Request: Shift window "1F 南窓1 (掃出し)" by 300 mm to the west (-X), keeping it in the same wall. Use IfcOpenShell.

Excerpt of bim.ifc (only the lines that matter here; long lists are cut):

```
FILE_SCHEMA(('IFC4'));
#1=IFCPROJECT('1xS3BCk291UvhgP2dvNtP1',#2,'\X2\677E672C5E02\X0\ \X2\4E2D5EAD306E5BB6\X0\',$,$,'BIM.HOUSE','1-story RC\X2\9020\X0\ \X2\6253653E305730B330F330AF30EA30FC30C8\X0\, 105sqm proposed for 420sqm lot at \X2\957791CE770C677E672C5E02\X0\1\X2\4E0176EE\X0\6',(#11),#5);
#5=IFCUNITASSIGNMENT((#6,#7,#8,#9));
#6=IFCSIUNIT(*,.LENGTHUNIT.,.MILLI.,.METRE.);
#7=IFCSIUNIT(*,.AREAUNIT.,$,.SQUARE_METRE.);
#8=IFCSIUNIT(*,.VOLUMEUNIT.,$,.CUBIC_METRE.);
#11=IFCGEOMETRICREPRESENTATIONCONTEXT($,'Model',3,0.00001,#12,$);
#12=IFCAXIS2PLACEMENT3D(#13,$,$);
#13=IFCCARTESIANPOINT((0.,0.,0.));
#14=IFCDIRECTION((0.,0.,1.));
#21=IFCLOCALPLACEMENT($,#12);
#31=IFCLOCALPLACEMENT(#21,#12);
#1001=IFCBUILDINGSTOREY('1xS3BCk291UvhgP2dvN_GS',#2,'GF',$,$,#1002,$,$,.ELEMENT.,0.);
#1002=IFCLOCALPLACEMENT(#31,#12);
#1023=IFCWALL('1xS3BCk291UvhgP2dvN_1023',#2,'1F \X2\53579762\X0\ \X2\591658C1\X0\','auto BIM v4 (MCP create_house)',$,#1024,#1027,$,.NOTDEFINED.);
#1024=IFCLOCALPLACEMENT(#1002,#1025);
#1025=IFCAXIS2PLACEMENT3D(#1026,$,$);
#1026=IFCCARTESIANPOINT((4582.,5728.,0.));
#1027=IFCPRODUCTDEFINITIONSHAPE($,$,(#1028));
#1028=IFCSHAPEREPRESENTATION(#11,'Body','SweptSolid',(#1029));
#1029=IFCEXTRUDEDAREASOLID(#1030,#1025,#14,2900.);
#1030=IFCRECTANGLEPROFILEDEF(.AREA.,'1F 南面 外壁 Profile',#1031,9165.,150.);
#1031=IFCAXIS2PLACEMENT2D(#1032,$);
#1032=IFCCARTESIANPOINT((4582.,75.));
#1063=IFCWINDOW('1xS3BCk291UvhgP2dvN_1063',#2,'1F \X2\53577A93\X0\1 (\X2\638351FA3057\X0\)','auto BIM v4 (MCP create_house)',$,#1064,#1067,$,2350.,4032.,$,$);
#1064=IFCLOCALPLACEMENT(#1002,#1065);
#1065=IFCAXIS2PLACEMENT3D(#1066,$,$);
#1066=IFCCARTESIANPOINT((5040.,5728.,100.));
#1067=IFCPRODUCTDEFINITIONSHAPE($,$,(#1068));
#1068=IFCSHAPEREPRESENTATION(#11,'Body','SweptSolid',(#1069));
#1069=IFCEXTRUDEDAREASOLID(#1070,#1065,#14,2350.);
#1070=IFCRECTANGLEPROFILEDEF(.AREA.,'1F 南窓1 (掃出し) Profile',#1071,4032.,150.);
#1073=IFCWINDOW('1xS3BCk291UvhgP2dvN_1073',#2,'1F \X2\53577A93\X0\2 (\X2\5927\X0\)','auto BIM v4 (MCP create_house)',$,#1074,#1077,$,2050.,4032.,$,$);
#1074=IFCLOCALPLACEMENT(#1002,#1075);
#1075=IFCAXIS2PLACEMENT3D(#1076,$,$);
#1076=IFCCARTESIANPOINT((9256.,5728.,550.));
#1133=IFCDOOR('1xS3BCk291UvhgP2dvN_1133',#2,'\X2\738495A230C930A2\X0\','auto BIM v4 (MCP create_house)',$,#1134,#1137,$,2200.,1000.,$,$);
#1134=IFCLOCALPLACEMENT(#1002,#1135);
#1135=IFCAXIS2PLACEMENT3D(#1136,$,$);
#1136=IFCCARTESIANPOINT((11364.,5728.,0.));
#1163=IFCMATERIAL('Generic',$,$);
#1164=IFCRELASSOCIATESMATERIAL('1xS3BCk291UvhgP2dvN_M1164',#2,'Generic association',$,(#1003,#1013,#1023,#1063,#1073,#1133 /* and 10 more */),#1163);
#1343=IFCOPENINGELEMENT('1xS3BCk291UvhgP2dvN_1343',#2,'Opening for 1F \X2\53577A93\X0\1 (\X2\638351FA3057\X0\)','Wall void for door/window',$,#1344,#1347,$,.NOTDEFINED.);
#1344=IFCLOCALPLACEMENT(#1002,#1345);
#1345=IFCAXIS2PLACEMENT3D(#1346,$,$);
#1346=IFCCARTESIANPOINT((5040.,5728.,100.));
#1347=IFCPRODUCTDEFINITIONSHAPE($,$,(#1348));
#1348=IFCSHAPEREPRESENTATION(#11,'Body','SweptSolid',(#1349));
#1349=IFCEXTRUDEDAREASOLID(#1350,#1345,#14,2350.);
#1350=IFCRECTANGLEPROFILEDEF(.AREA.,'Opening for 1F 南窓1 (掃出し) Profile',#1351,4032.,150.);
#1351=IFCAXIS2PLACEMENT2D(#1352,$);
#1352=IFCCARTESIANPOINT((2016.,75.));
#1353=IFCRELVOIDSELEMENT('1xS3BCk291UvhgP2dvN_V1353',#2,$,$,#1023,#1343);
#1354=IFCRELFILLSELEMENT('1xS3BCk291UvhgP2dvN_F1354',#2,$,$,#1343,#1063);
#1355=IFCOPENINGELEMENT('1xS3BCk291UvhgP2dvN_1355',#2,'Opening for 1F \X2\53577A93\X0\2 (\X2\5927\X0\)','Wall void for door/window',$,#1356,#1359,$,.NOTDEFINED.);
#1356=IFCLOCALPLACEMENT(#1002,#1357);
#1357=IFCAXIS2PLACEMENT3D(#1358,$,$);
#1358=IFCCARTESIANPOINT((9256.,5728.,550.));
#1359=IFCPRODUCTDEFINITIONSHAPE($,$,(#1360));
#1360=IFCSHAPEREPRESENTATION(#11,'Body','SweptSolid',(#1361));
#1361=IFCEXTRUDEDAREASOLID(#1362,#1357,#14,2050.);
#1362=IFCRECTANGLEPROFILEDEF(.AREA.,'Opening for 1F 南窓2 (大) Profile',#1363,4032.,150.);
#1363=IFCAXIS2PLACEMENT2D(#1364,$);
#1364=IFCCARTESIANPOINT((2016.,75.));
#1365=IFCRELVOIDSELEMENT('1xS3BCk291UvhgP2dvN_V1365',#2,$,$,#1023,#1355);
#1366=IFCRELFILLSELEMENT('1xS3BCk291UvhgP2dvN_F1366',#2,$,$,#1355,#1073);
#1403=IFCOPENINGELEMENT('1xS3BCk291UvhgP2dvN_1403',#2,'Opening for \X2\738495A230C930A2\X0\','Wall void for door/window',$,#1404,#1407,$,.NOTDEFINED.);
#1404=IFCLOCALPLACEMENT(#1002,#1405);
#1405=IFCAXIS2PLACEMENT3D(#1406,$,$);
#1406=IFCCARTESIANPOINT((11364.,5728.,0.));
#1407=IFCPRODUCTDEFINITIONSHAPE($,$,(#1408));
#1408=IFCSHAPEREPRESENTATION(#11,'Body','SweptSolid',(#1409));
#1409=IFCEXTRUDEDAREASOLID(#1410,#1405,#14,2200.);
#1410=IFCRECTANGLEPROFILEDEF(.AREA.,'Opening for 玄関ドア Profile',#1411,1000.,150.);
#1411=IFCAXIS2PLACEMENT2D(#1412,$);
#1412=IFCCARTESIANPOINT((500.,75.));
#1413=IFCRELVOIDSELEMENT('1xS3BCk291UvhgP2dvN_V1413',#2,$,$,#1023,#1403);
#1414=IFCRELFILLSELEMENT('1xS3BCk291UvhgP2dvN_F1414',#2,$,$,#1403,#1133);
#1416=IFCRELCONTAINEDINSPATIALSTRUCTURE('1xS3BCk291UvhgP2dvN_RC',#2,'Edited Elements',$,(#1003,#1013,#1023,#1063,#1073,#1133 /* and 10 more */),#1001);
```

```python
import ifcopenshell
import ifcopenshell.api.geometry
import ifcopenshell.util.placement
import ifcopenshell.util.unit

model = ifcopenshell.open("bim.ifc")
unit_scale = ifcopenshell.util.unit.calculate_unit_scale(model)

window = model.by_guid("1xS3BCk291UvhgP2dvN_1063")
opening = window.FillsVoids[0].RelatingOpeningElement
wall = opening.VoidsElements[0].RelatingBuildingElement

wall_matrix = ifcopenshell.util.placement.get_local_placement(wall.ObjectPlacement)
shift = wall_matrix[:3, 0] * -0.3 / unit_scale
before = ifcopenshell.util.placement.get_local_placement(window.ObjectPlacement)[:3, 3].copy()

# The window is not placed relative to its opening, so move both.
for product in (opening, window):
    matrix = ifcopenshell.util.placement.get_local_placement(product.ObjectPlacement)
    matrix[:3, 3] += shift
    ifcopenshell.api.geometry.edit_object_placement(model, product=product, matrix=matrix, is_si=False)

after = ifcopenshell.util.placement.get_local_placement(window.ObjectPlacement)[:3, 3]
print("window moved by", (after - before).round(3) + 0.0)

model.write("bim_edited.ifc")
```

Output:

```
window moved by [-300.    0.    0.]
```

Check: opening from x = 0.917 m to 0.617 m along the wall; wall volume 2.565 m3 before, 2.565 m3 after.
